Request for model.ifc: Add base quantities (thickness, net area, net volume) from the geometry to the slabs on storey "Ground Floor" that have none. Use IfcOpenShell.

First a look at what the model holds.

```python
import ifcopenshell
import ifcopenshell.util.element
import ifcopenshell.util.unit

model = ifcopenshell.open("model.ifc")
print(model.schema)
for unit_type in ("LENGTHUNIT", "AREAUNIT", "VOLUMEUNIT"):
    print(unit_type, ifcopenshell.util.unit.calculate_unit_scale(model, unit_type))
storey = next(s for s in model.by_type("IfcBuildingStorey") if s.Name == "Ground Floor")
slabs = [e for e in ifcopenshell.util.element.get_decomposition(storey) if e.is_a("IfcSlab")]
for e in sorted(slabs, key=lambda e: e.id()):
    print(e.id(), e.is_a(), e.Name, list(ifcopenshell.util.element.get_psets(e, qtos_only=True)), sep=" | ")
```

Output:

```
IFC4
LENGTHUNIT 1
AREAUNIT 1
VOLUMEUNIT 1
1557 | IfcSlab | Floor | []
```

```python
import ifcopenshell
import ifcopenshell.api.pset
import ifcopenshell.geom
import ifcopenshell.util.element
import ifcopenshell.util.shape
import ifcopenshell.util.unit

model = ifcopenshell.open("model.ifc")
unit_scale = ifcopenshell.util.unit.calculate_unit_scale(model)
area_scale = ifcopenshell.util.unit.calculate_unit_scale(model, "AREAUNIT")
volume_scale = ifcopenshell.util.unit.calculate_unit_scale(model, "VOLUMEUNIT")
settings = ifcopenshell.geom.settings()

storey = next(s for s in model.by_type("IfcBuildingStorey") if s.Name == "Ground Floor")
slabs = [e for e in ifcopenshell.util.element.get_decomposition(storey) if e.is_a("IfcSlab")]

for e in sorted(slabs, key=lambda e: e.id()):
    if ifcopenshell.util.element.get_psets(e, qtos_only=True, should_inherit=False):
        continue
    # Geometry comes back in metres, in the element's own axes.
    shape = ifcopenshell.geom.create_shape(settings, e)
    values = {
        "Width": ifcopenshell.util.shape.get_z(shape.geometry) / unit_scale,
        "NetArea": ifcopenshell.util.shape.get_footprint_area(shape.geometry) / area_scale,
        "NetVolume": ifcopenshell.util.shape.get_volume(shape.geometry) / volume_scale,
    }
    qto = ifcopenshell.api.pset.add_qto(model, product=e, name="Qto_SlabBaseQuantities")
    ifcopenshell.api.pset.edit_qto(model, qto=qto, properties=values)
    print(e.id(), {k: round(v, 3) for k, v in values.items()})

model.write("model_rev.ifc")
```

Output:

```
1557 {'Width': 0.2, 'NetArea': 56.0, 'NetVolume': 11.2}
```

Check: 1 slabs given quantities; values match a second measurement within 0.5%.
